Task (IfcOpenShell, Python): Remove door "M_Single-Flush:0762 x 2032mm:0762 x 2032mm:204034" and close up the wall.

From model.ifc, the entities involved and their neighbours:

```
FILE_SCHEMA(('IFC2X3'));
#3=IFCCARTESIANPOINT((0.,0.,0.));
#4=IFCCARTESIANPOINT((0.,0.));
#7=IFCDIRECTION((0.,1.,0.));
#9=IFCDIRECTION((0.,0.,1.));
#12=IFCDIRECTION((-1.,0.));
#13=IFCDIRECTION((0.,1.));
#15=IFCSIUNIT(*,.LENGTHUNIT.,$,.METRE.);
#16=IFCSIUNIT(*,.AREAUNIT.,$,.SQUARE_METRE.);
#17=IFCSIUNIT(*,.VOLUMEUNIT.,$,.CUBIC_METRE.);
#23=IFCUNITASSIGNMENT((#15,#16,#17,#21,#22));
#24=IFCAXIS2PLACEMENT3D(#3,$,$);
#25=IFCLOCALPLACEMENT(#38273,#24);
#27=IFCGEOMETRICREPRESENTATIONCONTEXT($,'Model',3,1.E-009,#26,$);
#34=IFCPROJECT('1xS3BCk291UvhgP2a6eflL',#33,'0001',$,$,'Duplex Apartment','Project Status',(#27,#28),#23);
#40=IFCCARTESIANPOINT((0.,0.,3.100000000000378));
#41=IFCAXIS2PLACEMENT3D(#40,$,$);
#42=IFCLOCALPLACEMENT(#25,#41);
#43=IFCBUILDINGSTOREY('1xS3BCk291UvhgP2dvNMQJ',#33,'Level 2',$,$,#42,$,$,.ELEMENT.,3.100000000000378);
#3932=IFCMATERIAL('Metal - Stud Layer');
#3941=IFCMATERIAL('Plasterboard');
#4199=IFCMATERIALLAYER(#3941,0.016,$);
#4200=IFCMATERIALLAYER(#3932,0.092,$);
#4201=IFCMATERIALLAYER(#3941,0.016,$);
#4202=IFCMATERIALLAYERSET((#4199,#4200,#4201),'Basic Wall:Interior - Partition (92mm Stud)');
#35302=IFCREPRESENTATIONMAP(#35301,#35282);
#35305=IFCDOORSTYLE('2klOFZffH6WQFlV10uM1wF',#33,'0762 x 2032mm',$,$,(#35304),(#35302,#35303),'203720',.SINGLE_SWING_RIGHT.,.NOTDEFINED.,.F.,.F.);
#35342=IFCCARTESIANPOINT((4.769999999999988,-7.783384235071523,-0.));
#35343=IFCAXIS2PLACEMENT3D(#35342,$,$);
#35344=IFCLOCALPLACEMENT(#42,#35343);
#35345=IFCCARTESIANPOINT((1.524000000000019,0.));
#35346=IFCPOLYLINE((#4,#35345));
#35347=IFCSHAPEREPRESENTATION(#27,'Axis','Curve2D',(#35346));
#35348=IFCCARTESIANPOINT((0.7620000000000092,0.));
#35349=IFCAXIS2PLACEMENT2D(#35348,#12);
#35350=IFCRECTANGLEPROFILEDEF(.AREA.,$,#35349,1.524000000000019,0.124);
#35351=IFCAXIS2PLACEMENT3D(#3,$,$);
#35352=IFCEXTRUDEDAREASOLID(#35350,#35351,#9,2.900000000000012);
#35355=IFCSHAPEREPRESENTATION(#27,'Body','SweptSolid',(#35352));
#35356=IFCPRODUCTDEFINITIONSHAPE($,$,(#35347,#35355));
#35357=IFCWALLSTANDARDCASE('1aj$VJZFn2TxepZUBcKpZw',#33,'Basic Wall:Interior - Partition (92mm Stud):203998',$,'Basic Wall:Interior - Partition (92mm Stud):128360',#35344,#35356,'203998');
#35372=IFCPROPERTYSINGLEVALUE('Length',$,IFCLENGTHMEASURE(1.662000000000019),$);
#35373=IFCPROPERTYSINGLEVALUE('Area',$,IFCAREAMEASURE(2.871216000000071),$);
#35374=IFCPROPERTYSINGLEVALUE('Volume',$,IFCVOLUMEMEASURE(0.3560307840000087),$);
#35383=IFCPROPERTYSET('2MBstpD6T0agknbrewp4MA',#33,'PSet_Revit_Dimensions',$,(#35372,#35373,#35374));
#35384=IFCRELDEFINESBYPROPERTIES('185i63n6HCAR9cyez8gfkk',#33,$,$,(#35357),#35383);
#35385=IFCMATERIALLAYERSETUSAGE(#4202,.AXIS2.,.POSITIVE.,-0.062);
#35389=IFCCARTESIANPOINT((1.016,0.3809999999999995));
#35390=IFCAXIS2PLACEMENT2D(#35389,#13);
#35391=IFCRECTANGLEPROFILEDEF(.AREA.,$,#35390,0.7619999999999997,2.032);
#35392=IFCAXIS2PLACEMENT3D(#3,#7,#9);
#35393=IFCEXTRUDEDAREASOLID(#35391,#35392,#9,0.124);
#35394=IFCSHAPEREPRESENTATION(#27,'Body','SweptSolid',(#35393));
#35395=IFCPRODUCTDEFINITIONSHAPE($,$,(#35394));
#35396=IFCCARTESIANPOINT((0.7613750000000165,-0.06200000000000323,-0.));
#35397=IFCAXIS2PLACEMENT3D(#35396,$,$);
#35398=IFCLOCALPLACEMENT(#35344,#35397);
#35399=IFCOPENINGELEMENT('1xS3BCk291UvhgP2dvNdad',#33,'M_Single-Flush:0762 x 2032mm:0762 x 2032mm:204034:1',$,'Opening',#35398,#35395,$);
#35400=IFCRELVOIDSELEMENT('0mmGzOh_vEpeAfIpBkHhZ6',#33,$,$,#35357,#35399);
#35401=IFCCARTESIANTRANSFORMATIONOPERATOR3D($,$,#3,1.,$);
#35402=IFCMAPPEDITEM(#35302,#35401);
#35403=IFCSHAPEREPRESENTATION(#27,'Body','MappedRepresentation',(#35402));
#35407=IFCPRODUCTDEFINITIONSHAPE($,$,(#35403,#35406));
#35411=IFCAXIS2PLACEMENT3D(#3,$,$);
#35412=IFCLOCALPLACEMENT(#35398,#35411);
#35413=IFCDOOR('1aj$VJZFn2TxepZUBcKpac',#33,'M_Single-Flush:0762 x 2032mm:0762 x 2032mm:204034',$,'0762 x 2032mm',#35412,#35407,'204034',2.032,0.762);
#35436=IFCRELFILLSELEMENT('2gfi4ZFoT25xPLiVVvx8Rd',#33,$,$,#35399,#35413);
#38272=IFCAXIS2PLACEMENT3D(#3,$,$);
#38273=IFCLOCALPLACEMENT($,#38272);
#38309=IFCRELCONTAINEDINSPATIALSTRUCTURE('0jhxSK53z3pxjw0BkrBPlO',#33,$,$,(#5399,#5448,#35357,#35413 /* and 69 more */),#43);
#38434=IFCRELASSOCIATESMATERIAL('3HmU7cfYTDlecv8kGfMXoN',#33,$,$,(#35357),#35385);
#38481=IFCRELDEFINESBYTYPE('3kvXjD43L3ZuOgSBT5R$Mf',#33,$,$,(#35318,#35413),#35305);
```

```python
import ifcopenshell
import ifcopenshell.api.feature
import ifcopenshell.api.pset
import ifcopenshell.api.root
import ifcopenshell.geom
import ifcopenshell.util.element
import ifcopenshell.util.shape
import ifcopenshell.util.unit

model = ifcopenshell.open("model.ifc")
area_scale = ifcopenshell.util.unit.calculate_unit_scale(model, "AREAUNIT")
volume_scale = ifcopenshell.util.unit.calculate_unit_scale(model, "VOLUMEUNIT")
settings = ifcopenshell.geom.settings()


def volume(element):
    """Net volume in cubic metres, openings subtracted."""
    shape = ifcopenshell.geom.create_shape(settings, element)
    return ifcopenshell.util.shape.get_volume(shape.geometry)


door = model.by_guid("1aj$VJZFn2TxepZUBcKpac")
opening = door.FillsVoids[0].RelatingOpeningElement
wall = opening.VoidsElements[0].RelatingBuildingElement
before = volume(wall)

ifcopenshell.api.root.remove_product(model, product=door)
ifcopenshell.api.feature.remove_feature(model, feature=opening)

after = volume(wall)
thickness = 0.124  # wall thickness in metres

# Update the wall's stored quantities.
pset = model.by_id(ifcopenshell.util.element.get_pset(wall, "PSet_Revit_Dimensions", should_inherit=False)["id"])
ifcopenshell.api.pset.edit_pset(model, pset=pset, properties={
    "Area": model.create_entity("IfcAreaMeasure", after / thickness / area_scale),
    "Volume": model.create_entity("IfcVolumeMeasure", after / volume_scale),
})

print(f"wall volume {before:.3f} -> {after:.3f} m3")

model.write("model-out.ifc")
```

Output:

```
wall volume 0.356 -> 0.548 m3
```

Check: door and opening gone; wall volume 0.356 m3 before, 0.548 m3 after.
